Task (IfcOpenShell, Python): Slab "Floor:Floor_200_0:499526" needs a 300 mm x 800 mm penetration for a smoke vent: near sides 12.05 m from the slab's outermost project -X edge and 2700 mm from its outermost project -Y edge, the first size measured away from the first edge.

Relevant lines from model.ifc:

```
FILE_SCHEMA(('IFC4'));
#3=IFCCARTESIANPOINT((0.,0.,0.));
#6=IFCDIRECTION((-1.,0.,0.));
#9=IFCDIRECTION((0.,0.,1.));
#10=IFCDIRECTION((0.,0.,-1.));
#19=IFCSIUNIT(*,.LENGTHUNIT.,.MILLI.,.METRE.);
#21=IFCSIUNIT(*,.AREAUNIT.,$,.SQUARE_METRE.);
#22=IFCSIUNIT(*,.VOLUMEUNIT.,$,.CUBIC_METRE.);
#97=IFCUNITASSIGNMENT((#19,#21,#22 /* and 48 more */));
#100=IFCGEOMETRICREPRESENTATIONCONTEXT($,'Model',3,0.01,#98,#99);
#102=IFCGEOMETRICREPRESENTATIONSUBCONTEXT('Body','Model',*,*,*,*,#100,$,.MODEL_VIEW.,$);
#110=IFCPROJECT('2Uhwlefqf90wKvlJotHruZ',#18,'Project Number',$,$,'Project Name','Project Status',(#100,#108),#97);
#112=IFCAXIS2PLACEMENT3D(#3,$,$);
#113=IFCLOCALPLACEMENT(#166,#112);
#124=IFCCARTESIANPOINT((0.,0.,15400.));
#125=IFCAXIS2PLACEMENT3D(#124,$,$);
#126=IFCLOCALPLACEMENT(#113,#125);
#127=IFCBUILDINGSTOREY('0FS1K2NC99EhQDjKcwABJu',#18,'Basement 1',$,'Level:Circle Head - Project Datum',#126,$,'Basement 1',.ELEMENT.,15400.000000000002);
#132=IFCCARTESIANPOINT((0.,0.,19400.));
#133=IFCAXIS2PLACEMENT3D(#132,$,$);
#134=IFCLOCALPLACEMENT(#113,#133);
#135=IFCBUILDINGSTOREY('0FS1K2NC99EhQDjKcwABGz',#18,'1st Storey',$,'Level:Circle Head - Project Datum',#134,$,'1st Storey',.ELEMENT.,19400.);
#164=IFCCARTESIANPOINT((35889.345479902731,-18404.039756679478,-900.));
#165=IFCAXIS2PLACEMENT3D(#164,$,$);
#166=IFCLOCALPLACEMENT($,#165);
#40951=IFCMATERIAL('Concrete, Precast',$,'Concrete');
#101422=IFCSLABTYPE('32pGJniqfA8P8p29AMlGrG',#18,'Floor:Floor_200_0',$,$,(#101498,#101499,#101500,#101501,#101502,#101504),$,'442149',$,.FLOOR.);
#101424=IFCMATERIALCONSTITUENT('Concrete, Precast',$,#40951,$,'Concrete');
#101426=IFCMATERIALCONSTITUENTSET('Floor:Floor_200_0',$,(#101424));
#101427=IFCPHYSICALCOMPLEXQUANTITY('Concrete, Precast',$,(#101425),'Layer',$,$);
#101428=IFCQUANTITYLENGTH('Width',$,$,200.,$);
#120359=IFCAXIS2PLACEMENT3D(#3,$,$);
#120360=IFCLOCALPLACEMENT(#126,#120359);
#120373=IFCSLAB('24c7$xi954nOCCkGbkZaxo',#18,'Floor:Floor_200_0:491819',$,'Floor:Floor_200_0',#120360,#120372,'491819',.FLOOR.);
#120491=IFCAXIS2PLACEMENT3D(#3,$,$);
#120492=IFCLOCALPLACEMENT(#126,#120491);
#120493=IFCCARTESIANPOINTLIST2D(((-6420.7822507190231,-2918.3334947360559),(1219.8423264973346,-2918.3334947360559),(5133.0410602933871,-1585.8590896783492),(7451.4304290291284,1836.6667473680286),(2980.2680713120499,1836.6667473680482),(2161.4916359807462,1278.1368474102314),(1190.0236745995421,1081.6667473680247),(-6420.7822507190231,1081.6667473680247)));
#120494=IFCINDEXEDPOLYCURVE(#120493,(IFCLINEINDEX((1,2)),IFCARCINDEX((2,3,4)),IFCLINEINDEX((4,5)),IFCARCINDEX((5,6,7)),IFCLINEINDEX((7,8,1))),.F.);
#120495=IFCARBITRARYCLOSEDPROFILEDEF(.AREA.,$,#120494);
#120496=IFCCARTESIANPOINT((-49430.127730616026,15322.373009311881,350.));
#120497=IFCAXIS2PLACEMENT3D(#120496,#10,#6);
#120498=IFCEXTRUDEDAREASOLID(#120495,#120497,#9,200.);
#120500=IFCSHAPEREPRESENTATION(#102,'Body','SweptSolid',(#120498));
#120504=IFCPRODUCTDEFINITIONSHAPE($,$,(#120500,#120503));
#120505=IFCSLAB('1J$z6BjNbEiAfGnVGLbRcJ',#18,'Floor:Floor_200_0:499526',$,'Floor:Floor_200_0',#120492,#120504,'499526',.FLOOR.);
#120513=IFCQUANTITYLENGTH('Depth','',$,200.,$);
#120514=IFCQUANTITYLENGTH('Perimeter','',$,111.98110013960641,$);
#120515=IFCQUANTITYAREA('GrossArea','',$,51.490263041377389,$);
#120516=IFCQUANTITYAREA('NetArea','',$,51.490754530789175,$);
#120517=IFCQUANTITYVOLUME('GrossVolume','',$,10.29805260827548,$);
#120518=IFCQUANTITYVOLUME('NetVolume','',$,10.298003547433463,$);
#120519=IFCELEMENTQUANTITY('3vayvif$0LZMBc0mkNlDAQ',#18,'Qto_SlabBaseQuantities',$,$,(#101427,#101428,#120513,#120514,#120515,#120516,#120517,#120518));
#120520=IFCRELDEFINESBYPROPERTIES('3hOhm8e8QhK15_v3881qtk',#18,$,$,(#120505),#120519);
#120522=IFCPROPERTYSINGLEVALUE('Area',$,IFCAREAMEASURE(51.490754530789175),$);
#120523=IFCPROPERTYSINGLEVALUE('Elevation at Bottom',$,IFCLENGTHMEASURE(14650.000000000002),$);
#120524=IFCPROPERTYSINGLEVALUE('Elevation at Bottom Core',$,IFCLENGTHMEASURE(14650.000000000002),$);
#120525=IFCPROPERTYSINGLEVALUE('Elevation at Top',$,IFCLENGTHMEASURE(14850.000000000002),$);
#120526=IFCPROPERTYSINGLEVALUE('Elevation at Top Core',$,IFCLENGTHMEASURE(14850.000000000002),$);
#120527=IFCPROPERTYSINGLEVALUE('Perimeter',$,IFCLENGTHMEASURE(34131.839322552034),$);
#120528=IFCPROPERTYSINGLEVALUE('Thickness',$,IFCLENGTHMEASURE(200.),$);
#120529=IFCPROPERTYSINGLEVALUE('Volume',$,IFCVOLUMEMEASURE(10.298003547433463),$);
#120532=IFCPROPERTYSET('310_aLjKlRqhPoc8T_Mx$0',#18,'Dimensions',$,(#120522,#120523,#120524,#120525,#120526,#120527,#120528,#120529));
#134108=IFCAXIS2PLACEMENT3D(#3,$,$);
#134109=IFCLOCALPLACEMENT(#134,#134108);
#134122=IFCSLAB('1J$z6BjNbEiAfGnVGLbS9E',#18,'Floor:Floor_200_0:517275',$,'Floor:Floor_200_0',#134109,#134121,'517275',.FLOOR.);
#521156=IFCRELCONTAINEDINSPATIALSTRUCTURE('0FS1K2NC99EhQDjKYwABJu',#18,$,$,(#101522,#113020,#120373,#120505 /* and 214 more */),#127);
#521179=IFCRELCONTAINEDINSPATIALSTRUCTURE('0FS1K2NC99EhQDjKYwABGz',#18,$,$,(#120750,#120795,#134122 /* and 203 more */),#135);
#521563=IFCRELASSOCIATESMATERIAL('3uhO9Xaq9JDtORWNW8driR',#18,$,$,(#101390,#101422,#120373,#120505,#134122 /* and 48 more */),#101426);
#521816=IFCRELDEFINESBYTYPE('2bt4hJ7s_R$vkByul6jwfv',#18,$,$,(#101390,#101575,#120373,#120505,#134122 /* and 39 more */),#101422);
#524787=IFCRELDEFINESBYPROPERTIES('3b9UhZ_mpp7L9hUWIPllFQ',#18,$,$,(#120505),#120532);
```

```python
import numpy as np
import ifcopenshell
import ifcopenshell.api.feature
import ifcopenshell.api.geometry
import ifcopenshell.api.pset
import ifcopenshell.api.root
import ifcopenshell.geom
import ifcopenshell.util.element
import ifcopenshell.util.placement
import ifcopenshell.util.representation
import ifcopenshell.util.shape
import ifcopenshell.util.unit

model = ifcopenshell.open("model.ifc")
unit_scale = ifcopenshell.util.unit.calculate_unit_scale(model)
area_scale = ifcopenshell.util.unit.calculate_unit_scale(model, "AREAUNIT")
volume_scale = ifcopenshell.util.unit.calculate_unit_scale(model, "VOLUMEUNIT")
settings = ifcopenshell.geom.settings()


def volume(element):
    """Net volume in cubic metres, openings subtracted."""
    shape = ifcopenshell.geom.create_shape(settings, element)
    return ifcopenshell.util.shape.get_volume(shape.geometry)


slab = model.by_guid("1J$z6BjNbEiAfGnVGLbRcJ")
before = volume(slab)

# Extent in the slab's own axes, in metres. The edges named are its -X and -Y sides.
slab_shape = ifcopenshell.geom.create_shape(settings, slab)
vertices = ifcopenshell.util.shape.get_vertices(slab_shape.geometry)
x_min, y_min, bottom = vertices.min(axis=0)
top = vertices[:, 2].max()

opening = ifcopenshell.api.root.create_entity(model, ifc_class="IfcOpeningElement", name="Smoke vent opening", predefined_type="OPENING")
context = ifcopenshell.util.representation.get_context(model, "Model", "Body", "MODEL_VIEW")
width, depth = 0.3, 0.8
outline = [(0.0, 0.0), (width, 0.0), (width, depth), (0.0, depth), (0.0, 0.0)]
# Overshoot both faces by 50 mm so the cut is clean.
shape = ifcopenshell.api.geometry.add_slab_representation(
    model, context=context, depth=top - bottom + 0.1, polyline=outline
)
ifcopenshell.api.geometry.assign_representation(model, product=opening, representation=shape)

matrix = ifcopenshell.util.placement.get_local_placement(slab.ObjectPlacement)
matrix[:, 3] = matrix @ np.append(np.array([x_min + 12.05, y_min + 2.7, bottom - 0.05]) / unit_scale, 1.0)
ifcopenshell.api.geometry.edit_object_placement(model, product=opening, matrix=matrix, is_si=False)
ifcopenshell.api.feature.add_feature(model, feature=opening, element=slab)

after = volume(slab)

# Update the slab's stored quantities.
qto = model.by_id(ifcopenshell.util.element.get_pset(slab, "Qto_SlabBaseQuantities", should_inherit=False)["id"])
ifcopenshell.api.pset.edit_qto(model, qto=qto, properties={
    "NetArea": after / (top - bottom) / area_scale,
    "NetVolume": after / volume_scale,
})
pset = model.by_id(ifcopenshell.util.element.get_pset(slab, "Dimensions", should_inherit=False)["id"])
ifcopenshell.api.pset.edit_pset(model, pset=pset, properties={
    "Area": model.create_entity("IfcAreaMeasure", after / (top - bottom) / area_scale),
    "Volume": model.create_entity("IfcVolumeMeasure", after / volume_scale),
})

print(f"slab volume {before:.3f} -> {after:.3f} m3")

model.write("model_rev.ifc")
```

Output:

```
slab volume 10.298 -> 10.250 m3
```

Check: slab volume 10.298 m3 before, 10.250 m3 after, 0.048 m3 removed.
